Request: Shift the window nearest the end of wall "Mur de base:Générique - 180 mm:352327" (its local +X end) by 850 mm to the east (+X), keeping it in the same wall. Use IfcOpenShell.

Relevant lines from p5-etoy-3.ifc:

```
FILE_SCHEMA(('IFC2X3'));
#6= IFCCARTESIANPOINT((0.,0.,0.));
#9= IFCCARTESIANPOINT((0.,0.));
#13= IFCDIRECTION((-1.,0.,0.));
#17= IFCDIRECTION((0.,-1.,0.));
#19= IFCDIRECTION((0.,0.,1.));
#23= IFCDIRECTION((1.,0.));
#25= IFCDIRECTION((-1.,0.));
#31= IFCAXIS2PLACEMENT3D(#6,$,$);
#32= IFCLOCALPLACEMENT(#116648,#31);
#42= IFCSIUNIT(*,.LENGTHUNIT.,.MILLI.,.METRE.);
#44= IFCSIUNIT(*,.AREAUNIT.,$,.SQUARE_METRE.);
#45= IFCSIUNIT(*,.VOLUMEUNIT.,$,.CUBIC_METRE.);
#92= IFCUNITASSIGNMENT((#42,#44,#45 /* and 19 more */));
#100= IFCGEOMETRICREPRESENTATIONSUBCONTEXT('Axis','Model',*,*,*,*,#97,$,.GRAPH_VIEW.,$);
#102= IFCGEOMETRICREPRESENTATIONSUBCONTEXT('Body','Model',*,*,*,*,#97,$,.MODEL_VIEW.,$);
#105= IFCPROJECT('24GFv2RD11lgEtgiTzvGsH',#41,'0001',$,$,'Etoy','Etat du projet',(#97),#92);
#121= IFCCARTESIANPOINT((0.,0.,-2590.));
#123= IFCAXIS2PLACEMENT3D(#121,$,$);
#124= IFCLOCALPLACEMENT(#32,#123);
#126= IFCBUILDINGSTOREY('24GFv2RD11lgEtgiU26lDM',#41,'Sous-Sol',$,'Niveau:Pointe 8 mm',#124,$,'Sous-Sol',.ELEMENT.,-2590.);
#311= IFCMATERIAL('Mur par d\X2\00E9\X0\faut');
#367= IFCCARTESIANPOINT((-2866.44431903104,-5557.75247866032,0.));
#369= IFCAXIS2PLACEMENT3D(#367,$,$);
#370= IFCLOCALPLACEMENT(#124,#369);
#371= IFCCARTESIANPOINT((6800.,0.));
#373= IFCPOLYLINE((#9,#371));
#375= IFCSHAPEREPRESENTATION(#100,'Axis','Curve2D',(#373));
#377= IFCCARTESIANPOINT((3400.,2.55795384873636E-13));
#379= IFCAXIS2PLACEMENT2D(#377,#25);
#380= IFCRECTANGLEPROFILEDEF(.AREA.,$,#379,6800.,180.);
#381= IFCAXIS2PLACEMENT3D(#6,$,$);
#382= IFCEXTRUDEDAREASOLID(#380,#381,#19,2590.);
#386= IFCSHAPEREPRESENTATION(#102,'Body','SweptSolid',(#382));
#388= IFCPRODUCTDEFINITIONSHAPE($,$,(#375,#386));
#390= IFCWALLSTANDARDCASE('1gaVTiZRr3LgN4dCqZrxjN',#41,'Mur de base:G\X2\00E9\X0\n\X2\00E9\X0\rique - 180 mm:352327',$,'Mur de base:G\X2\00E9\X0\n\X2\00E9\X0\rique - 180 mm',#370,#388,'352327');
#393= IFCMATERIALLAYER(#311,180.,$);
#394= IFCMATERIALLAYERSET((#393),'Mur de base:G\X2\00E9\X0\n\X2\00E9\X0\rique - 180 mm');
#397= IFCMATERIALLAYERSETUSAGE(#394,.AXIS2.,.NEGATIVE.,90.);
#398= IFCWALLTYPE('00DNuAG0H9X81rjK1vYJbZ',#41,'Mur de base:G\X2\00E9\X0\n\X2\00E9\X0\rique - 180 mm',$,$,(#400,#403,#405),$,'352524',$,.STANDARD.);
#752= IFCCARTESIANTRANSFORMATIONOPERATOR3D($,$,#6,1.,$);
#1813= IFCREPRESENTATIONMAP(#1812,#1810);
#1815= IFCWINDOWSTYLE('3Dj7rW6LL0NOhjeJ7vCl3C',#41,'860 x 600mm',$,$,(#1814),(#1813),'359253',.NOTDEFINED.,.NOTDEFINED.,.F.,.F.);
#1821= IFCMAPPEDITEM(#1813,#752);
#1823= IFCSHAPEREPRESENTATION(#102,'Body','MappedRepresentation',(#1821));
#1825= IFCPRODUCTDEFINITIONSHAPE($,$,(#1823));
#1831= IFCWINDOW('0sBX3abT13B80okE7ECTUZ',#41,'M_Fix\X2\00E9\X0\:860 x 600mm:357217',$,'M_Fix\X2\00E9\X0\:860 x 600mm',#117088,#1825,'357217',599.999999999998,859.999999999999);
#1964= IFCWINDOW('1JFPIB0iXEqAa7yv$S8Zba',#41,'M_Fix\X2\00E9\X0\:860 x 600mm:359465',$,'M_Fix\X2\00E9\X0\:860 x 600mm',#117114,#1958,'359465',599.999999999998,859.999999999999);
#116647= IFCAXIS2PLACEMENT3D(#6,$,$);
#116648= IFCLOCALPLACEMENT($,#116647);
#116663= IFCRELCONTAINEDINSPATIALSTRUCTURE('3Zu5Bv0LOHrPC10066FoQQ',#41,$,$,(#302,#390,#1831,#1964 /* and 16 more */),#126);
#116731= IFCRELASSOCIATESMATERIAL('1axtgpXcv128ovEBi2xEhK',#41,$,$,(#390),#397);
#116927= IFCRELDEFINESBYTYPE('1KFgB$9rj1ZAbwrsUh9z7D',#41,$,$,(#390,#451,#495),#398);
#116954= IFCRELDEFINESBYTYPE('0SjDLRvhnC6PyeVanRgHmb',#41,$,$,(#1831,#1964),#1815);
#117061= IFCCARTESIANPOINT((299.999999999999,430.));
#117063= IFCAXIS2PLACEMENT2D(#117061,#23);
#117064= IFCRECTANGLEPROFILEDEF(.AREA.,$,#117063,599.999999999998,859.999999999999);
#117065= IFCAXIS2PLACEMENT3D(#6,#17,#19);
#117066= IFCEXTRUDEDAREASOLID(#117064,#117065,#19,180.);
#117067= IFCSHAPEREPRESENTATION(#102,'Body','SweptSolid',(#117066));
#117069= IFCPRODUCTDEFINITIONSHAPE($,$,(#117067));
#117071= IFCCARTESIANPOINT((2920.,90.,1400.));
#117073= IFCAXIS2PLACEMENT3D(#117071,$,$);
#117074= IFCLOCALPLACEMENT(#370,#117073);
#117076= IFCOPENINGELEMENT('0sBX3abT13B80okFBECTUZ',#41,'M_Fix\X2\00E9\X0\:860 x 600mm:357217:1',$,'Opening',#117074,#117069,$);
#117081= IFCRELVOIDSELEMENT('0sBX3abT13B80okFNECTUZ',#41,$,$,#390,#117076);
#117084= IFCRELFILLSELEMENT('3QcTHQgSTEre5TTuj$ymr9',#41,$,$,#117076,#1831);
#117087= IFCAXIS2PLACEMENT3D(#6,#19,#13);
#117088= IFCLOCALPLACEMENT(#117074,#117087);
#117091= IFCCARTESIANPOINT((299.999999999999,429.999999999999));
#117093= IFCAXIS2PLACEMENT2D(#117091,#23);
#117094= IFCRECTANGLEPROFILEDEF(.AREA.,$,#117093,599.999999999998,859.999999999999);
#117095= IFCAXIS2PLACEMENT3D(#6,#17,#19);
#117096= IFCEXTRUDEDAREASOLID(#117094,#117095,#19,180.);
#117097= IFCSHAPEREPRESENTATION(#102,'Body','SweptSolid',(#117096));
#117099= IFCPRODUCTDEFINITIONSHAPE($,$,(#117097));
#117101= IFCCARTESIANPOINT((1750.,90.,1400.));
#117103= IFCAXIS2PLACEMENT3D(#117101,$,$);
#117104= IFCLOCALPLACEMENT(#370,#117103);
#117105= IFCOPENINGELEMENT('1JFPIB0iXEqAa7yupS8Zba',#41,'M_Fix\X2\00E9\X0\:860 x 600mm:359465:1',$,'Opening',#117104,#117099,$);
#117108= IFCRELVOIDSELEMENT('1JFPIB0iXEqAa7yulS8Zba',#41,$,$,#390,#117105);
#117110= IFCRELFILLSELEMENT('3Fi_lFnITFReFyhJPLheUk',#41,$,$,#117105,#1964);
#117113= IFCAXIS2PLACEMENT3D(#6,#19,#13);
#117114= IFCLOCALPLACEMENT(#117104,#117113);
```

```python
import ifcopenshell
import ifcopenshell.api.geometry
import ifcopenshell.util.placement
import ifcopenshell.util.unit

model = ifcopenshell.open("p5-etoy-3.ifc")
unit_scale = ifcopenshell.util.unit.calculate_unit_scale(model)

window = model.by_guid("0sBX3abT13B80okE7ECTUZ")
opening = window.FillsVoids[0].RelatingOpeningElement
wall = opening.VoidsElements[0].RelatingBuildingElement

wall_matrix = ifcopenshell.util.placement.get_local_placement(wall.ObjectPlacement)
shift = wall_matrix[:3, 0] * 0.85 / unit_scale
before = ifcopenshell.util.placement.get_local_placement(window.ObjectPlacement)[:3, 3].copy()

# The window is placed relative to its opening, so it follows when the opening moves.
matrix = ifcopenshell.util.placement.get_local_placement(opening.ObjectPlacement)
matrix[:3, 3] += shift
ifcopenshell.api.geometry.edit_object_placement(
    model, product=opening, matrix=matrix, is_si=False, should_transform_children=True
)

after = ifcopenshell.util.placement.get_local_placement(window.ObjectPlacement)[:3, 3]
print("window moved by", (after - before).round(3) + 0.0)

model.write("p5-etoy-3-out.ifc")
```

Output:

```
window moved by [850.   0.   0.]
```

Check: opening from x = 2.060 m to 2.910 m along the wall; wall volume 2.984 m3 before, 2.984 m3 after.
